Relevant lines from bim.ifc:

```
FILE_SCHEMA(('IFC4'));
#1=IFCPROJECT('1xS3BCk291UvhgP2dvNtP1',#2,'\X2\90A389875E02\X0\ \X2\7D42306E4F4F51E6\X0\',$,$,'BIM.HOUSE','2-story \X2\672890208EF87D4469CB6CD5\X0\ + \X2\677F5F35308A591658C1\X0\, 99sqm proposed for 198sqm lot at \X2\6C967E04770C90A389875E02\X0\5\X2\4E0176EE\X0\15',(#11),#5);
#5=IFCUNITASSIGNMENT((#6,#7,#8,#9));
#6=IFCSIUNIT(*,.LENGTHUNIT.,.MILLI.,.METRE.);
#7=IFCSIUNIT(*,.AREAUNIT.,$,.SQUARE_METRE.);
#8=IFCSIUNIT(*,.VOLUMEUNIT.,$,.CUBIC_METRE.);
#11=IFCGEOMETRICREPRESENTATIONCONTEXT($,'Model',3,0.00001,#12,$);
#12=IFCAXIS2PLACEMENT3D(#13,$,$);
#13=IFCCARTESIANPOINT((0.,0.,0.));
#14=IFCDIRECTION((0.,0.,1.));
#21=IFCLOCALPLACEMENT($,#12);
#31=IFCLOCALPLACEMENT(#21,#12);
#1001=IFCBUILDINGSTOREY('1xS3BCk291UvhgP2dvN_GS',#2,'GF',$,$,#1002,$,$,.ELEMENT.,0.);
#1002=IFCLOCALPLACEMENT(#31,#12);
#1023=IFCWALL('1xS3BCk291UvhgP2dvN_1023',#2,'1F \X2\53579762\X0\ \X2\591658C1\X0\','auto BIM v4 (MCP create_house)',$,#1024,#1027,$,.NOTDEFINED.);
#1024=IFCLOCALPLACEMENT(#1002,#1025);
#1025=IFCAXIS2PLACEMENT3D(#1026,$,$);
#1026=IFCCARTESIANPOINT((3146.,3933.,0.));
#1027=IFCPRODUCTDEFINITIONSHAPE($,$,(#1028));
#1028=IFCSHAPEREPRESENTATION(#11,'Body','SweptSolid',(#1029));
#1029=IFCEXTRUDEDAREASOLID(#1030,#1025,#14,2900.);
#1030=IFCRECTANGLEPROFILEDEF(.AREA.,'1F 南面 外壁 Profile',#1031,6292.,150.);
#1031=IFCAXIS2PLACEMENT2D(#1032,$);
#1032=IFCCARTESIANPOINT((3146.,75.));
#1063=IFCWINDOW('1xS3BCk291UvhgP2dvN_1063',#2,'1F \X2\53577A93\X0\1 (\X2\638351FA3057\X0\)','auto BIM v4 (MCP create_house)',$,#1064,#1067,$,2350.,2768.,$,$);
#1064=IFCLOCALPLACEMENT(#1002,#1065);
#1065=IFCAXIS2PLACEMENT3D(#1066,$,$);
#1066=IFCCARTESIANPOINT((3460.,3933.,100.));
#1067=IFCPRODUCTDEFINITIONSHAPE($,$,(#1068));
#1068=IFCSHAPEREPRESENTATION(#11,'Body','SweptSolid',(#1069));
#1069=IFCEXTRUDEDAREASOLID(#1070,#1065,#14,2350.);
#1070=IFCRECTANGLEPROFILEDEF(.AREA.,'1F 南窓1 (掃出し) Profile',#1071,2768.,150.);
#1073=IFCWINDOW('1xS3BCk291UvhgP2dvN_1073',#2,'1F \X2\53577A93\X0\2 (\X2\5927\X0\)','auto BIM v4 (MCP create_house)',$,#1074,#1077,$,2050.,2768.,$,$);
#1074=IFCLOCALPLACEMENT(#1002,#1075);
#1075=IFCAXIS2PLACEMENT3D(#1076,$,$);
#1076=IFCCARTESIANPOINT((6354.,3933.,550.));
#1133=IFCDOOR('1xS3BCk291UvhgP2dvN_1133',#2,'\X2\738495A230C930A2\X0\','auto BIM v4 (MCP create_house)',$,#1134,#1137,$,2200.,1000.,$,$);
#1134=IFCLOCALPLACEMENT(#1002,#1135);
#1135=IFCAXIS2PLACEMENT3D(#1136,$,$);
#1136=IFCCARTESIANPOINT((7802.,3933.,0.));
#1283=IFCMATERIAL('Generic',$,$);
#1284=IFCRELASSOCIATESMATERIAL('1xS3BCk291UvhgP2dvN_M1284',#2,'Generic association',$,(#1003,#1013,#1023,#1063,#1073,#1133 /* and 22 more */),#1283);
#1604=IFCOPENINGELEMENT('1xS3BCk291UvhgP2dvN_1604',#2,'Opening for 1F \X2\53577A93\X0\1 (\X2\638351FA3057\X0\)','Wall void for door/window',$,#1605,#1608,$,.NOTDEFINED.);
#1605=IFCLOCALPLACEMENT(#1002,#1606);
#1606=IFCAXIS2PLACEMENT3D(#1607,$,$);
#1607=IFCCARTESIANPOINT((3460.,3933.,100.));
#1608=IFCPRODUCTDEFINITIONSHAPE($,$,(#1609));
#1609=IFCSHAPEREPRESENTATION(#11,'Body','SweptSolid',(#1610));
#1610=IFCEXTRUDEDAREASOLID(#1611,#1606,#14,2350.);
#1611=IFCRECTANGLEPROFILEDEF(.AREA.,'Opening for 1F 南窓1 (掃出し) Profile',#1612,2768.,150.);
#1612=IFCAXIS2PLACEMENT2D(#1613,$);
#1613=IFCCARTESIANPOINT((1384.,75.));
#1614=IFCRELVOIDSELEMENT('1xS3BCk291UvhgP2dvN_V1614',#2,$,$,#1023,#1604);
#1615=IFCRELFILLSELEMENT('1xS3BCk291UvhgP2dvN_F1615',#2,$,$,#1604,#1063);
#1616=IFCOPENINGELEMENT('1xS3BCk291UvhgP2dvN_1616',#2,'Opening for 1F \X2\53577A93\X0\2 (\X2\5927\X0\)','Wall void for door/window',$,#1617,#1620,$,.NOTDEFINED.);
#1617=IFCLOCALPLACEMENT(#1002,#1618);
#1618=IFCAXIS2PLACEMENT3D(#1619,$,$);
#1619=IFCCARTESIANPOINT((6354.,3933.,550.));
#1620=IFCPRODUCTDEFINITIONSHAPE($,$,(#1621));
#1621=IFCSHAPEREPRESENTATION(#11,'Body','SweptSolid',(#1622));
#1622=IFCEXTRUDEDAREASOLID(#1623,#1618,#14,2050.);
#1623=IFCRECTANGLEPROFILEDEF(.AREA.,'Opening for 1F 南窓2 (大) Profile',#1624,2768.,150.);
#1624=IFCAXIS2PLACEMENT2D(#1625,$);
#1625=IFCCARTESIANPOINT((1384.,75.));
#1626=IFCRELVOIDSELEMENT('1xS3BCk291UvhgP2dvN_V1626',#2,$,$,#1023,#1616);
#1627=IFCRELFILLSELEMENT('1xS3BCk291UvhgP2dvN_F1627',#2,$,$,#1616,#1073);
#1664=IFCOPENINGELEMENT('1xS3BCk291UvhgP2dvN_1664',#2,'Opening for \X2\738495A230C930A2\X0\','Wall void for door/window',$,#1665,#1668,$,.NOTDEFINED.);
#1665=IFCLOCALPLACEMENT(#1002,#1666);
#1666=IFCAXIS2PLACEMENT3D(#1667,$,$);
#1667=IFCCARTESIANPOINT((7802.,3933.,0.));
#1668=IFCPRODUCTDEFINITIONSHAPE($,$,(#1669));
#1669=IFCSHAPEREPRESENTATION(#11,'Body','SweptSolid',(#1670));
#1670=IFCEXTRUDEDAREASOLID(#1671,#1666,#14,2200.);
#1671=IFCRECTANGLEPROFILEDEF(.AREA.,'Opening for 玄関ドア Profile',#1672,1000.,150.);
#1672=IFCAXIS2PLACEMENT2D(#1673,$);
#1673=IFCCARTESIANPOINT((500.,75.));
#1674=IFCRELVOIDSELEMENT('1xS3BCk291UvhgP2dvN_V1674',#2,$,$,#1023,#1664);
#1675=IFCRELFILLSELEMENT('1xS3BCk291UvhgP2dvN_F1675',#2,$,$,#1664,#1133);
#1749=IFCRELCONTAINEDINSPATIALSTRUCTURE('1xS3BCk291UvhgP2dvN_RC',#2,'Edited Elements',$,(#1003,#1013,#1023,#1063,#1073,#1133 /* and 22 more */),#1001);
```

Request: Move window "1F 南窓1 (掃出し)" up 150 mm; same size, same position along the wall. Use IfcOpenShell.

```python
import numpy as np
import ifcopenshell
import ifcopenshell.api.geometry
import ifcopenshell.util.placement
import ifcopenshell.util.unit

model = ifcopenshell.open("bim.ifc")
unit_scale = ifcopenshell.util.unit.calculate_unit_scale(model)

window = model.by_id(1063)
opening = window.FillsVoids[0].RelatingOpeningElement
dz = 0.15 / unit_scale

shift = np.array([0.0, 0.0, dz])
# The window is not placed relative to its opening, so move both.
for product in (opening, window):
    matrix = ifcopenshell.util.placement.get_local_placement(product.ObjectPlacement)
    matrix[:3, 3] += shift
    ifcopenshell.api.geometry.edit_object_placement(model, product=product, matrix=matrix, is_si=False)

print(f"moved by {dz * unit_scale:+.3f} m")

model.write("bim_v2.ifc")
```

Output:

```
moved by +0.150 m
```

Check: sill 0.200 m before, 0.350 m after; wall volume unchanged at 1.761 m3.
